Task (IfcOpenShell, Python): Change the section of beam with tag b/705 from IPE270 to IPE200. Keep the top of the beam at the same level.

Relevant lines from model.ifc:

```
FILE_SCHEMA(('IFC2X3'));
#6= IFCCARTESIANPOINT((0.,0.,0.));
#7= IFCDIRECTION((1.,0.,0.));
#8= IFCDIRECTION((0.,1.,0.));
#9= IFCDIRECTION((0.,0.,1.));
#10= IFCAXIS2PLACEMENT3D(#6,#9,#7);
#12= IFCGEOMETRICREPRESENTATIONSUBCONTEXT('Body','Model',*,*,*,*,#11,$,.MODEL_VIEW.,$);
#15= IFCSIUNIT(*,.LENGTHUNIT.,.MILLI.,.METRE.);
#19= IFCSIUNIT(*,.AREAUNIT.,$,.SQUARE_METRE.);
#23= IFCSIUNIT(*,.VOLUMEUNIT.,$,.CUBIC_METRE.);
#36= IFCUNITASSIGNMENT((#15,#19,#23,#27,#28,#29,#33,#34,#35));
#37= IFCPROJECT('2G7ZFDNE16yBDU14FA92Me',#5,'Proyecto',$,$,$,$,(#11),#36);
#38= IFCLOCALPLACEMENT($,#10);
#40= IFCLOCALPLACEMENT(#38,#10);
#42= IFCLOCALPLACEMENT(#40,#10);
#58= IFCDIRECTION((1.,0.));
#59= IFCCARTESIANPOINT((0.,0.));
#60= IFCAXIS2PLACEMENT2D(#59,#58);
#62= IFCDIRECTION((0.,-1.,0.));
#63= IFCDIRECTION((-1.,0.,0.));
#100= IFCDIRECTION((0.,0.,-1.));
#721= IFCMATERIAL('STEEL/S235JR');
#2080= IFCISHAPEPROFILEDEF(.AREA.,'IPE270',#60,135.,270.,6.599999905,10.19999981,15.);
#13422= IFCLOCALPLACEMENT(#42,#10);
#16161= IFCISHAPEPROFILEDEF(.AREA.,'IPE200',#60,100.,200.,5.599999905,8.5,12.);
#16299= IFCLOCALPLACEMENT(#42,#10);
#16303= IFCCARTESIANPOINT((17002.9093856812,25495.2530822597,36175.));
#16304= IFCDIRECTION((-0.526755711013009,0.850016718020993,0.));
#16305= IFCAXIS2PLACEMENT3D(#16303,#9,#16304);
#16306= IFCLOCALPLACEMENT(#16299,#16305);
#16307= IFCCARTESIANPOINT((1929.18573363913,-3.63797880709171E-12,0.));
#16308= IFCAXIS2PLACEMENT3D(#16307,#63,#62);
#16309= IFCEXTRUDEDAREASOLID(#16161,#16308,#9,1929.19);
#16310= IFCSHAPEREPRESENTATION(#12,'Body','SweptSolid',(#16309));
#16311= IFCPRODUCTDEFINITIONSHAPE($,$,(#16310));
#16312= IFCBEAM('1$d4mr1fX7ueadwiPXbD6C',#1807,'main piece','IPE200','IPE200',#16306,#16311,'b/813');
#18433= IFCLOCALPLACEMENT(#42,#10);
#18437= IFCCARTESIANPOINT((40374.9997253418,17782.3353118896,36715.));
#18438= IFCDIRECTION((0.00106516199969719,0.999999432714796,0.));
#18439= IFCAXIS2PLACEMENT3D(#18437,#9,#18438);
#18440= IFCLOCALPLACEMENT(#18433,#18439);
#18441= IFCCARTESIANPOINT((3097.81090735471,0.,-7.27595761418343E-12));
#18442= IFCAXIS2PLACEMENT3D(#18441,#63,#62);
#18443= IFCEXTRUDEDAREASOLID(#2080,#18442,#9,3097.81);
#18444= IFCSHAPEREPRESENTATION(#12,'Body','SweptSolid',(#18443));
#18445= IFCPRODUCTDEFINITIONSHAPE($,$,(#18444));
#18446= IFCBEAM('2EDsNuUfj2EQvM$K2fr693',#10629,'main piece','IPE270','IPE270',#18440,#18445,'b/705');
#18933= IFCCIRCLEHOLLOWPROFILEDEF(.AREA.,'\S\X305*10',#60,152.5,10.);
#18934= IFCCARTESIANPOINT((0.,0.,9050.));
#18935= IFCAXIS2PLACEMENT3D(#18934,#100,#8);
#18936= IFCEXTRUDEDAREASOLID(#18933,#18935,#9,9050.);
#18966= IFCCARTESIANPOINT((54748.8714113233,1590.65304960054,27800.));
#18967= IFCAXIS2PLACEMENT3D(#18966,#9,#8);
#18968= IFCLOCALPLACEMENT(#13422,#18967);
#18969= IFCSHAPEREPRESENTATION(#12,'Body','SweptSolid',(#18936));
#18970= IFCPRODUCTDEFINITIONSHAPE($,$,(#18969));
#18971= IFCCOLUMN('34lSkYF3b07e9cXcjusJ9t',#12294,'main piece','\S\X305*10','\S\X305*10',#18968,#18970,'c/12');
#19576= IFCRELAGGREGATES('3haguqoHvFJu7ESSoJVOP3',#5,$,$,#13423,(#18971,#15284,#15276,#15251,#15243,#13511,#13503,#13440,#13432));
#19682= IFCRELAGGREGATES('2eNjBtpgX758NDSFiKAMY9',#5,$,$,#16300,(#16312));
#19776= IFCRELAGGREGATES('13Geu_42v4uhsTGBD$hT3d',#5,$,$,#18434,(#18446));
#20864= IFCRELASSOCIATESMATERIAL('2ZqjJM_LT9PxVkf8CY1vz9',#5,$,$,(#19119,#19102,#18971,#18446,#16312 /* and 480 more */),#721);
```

```python
import ifcopenshell
import ifcopenshell.util.element
import ifcopenshell.util.representation

model = ifcopenshell.open("model.ifc")

member = model.by_guid("2EDsNuUfj2EQvM$K2fr693")
source = next(p for p in model.by_type("IfcIShapeProfileDef") if p.ProfileName == "IPE200")

body = ifcopenshell.util.representation.get_representation(member, "Model", "Body")
solid = body.Items[0]
old_profile = solid.SweptArea

# Copy the section's sizes but keep this member's own profile position.
profile = ifcopenshell.util.element.copy(model, source)
# Profiles are centred, so shift by half the change in depth to hold the top.
shift = (old_profile.OverallDepth - profile.OverallDepth) / 2
x, y = old_profile.Position.Location.Coordinates
up = (0.0, 1.0)  # upwards, in the solid's own plane
location = model.createIfcCartesianPoint((x + up[0] * shift, y + up[1] * shift))
profile.Position = model.createIfcAxis2Placement2D(location, old_profile.Position.RefDirection)
solid.SweptArea = profile
if not model.get_total_inverses(old_profile):
    ifcopenshell.util.element.remove_deep2(model, old_profile)
member.Description = member.Description.replace("IPE270", "IPE200")
member.ObjectType = member.ObjectType.replace("IPE270", "IPE200")

print(solid.SweptArea)

model.write("model_v2.ifc")
```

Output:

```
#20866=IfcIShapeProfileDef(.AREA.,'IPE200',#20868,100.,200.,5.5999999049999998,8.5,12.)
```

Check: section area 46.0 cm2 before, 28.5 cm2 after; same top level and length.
